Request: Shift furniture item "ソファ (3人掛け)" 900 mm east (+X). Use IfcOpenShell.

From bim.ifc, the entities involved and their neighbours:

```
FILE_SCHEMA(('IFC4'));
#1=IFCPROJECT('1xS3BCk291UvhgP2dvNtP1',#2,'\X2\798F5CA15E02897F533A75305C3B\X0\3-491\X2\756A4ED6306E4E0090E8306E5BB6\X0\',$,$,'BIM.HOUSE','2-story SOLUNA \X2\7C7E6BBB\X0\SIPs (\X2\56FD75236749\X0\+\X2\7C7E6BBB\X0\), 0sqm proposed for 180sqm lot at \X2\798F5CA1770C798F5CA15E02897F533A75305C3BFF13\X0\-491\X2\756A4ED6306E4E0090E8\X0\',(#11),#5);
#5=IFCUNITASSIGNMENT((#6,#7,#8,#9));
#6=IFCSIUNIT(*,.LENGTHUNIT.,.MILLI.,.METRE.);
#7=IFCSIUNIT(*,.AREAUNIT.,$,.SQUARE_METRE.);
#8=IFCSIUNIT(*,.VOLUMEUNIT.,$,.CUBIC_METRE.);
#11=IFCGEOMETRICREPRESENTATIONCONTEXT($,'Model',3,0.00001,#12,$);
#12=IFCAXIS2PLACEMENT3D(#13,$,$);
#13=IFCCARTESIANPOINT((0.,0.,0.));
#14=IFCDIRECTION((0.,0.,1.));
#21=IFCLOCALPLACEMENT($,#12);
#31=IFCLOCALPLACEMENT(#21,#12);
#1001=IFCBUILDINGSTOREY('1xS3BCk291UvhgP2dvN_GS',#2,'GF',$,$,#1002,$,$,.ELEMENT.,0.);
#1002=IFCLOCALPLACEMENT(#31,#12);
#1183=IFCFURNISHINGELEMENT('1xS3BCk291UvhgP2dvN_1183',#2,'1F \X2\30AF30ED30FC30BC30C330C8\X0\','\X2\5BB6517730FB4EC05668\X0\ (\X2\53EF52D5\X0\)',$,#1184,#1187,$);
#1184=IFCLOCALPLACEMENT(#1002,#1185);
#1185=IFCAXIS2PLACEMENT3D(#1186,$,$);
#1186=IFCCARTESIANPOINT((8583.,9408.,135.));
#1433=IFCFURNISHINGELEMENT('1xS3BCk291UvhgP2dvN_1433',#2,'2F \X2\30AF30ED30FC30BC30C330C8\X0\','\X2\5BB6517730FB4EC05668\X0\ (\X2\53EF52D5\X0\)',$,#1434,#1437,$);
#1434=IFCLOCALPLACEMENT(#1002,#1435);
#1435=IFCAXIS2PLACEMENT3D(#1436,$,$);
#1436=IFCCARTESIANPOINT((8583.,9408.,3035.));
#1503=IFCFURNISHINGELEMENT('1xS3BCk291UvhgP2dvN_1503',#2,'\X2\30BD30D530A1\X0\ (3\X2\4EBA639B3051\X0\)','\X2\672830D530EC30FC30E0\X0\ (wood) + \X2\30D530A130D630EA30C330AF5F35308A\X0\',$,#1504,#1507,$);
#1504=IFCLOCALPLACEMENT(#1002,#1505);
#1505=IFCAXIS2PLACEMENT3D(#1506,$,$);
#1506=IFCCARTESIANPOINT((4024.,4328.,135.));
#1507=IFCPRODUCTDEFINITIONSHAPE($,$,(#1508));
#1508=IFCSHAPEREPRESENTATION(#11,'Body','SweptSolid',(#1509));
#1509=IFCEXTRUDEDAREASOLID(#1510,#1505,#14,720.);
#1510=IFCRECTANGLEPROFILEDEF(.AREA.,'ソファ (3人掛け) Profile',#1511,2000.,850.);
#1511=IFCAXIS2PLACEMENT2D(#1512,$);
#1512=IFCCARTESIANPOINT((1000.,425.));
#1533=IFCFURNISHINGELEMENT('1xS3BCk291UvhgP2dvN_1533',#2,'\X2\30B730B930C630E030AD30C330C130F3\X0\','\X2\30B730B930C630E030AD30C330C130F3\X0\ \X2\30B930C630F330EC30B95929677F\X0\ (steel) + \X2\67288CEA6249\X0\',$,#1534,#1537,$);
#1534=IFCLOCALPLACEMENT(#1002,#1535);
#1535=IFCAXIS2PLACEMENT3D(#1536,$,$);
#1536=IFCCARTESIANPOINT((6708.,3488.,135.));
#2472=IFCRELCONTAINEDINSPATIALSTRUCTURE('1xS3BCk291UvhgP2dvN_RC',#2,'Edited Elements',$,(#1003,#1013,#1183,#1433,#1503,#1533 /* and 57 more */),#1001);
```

```python
import ifcopenshell
import ifcopenshell.api.geometry
import ifcopenshell.util.placement
import ifcopenshell.util.unit

model = ifcopenshell.open("bim.ifc")
unit_scale = ifcopenshell.util.unit.calculate_unit_scale(model)

item = model.by_guid("1xS3BCk291UvhgP2dvN_1503")
matrix = ifcopenshell.util.placement.get_local_placement(item.ObjectPlacement)
matrix[0, 3] += 0.9 / unit_scale
ifcopenshell.api.geometry.edit_object_placement(model, product=item, matrix=matrix, is_si=False)

print(ifcopenshell.util.placement.get_local_placement(item.ObjectPlacement).round(3) + 0.0)

model.write("bim_rev.ifc")
```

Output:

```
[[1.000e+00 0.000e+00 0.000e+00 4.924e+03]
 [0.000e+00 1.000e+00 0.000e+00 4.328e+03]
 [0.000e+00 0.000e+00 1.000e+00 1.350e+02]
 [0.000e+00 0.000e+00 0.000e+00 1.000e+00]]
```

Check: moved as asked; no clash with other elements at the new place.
